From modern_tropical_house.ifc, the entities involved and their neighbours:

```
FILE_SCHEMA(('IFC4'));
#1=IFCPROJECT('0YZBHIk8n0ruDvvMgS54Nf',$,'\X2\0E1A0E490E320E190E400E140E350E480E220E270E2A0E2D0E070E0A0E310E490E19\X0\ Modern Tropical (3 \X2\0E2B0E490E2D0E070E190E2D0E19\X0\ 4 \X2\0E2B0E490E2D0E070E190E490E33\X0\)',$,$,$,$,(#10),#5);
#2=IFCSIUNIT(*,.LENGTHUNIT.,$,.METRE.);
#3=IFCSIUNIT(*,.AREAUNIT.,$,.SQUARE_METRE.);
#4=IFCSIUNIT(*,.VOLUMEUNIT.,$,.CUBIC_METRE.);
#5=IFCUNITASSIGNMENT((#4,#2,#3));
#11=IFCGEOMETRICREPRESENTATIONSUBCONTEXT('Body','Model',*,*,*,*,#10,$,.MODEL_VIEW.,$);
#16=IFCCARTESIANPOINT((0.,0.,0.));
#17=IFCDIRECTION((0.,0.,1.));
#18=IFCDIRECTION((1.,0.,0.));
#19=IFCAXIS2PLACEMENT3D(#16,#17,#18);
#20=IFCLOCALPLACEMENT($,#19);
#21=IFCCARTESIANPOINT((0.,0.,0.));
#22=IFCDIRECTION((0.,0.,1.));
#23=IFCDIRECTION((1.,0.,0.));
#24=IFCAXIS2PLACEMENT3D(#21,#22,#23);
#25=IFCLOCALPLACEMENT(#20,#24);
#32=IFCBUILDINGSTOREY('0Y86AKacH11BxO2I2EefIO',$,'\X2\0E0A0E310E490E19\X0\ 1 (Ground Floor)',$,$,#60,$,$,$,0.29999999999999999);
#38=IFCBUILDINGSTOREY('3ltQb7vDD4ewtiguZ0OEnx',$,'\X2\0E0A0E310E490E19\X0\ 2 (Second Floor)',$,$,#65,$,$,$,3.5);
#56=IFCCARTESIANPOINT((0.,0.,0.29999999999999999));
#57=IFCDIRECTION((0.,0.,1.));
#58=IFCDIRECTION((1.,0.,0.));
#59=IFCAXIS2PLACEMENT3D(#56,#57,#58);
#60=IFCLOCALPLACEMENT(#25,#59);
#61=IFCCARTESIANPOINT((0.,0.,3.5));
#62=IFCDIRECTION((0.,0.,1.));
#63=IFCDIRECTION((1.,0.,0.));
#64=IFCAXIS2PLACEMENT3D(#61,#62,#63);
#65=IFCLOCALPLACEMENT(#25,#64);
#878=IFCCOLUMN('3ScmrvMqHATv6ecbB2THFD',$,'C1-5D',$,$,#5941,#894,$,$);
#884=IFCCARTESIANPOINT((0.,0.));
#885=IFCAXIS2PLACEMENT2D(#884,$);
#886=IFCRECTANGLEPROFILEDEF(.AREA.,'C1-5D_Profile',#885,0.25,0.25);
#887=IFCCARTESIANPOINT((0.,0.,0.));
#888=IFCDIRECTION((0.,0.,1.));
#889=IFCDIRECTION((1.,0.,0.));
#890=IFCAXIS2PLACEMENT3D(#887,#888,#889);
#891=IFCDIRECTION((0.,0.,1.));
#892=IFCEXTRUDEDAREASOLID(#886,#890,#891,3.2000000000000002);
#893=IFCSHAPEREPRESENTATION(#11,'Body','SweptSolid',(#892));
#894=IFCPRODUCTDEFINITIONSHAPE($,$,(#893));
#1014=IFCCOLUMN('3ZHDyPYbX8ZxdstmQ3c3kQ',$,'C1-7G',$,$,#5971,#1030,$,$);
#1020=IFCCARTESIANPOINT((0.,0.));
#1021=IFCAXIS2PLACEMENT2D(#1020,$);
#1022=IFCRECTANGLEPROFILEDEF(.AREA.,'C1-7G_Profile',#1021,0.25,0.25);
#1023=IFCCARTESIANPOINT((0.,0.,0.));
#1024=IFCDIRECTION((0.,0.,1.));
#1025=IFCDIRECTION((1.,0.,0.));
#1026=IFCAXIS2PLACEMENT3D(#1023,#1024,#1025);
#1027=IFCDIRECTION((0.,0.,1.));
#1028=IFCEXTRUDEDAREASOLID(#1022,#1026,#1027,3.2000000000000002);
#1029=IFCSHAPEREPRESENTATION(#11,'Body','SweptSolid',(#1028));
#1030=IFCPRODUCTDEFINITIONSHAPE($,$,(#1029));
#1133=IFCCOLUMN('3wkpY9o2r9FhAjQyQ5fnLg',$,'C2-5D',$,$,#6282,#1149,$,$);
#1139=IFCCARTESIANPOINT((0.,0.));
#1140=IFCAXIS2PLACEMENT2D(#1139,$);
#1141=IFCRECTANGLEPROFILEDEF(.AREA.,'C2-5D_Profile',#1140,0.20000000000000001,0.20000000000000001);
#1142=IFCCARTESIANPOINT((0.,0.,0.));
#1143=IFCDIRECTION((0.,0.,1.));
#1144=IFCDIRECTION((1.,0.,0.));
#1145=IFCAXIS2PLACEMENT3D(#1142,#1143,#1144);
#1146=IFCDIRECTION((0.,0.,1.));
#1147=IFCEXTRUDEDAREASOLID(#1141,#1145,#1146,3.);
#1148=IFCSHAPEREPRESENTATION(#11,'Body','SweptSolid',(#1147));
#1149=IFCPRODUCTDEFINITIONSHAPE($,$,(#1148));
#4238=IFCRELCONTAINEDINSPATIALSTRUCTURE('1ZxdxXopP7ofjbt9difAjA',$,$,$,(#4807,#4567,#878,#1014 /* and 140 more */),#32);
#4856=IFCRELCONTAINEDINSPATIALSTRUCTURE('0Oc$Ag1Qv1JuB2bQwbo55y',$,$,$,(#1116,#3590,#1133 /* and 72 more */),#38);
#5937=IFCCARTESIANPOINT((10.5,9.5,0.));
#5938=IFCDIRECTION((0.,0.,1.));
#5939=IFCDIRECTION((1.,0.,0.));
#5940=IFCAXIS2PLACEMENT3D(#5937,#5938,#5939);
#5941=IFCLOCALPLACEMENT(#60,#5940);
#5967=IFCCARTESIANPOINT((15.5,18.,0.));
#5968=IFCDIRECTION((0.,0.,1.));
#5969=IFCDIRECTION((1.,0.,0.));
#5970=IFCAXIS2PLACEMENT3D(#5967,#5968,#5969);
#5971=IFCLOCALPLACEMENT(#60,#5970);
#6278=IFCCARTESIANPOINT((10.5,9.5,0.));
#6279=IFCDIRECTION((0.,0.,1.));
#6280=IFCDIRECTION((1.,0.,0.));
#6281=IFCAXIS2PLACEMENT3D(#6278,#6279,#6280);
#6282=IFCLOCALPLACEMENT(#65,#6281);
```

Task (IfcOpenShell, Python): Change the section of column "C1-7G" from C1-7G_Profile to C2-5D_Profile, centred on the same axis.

```python
import ifcopenshell
import ifcopenshell.util.element
import ifcopenshell.util.representation

model = ifcopenshell.open("modern_tropical_house.ifc")

member = model.by_guid("3ZHDyPYbX8ZxdstmQ3c3kQ")
source = next(p for p in model.by_type("IfcRectangleProfileDef") if p.ProfileName == "C2-5D_Profile")

body = ifcopenshell.util.representation.get_representation(member, "Model", "Body")
solid = body.Items[0]
old_profile = solid.SweptArea

# Copy the section's sizes but keep this member's own profile position.
profile = ifcopenshell.util.element.copy(model, source)
profile.Position = old_profile.Position
solid.SweptArea = profile
if not model.get_total_inverses(old_profile):
    ifcopenshell.util.element.remove_deep2(model, old_profile)

print(solid.SweptArea)

model.write("modern_tropical_house_updated.ifc")
```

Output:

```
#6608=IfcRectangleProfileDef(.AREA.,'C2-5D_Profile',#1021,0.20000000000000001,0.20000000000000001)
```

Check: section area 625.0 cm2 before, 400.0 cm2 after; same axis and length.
